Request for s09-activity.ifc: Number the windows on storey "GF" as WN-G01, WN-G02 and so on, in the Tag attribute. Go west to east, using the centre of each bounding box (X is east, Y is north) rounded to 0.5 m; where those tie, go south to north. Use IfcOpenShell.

First a look at what the model holds.

```python
import ifcopenshell
import ifcopenshell.util.element
import ifcopenshell.util.placement

model = ifcopenshell.open("s09-activity.ifc")
print(model.schema)
storey = next(s for s in model.by_type("IfcBuildingStorey") if s.Name == "GF")
windows = [e for e in ifcopenshell.util.element.get_decomposition(storey) if e.is_a("IfcWindow")]
for e in sorted(windows, key=lambda e: e.id()):
    origin = ifcopenshell.util.placement.get_local_placement(e.ObjectPlacement)[:3, 3]
    print(e.id(), e.Tag, e.Name, origin.round(2) + 0.0, sep=" | ")
```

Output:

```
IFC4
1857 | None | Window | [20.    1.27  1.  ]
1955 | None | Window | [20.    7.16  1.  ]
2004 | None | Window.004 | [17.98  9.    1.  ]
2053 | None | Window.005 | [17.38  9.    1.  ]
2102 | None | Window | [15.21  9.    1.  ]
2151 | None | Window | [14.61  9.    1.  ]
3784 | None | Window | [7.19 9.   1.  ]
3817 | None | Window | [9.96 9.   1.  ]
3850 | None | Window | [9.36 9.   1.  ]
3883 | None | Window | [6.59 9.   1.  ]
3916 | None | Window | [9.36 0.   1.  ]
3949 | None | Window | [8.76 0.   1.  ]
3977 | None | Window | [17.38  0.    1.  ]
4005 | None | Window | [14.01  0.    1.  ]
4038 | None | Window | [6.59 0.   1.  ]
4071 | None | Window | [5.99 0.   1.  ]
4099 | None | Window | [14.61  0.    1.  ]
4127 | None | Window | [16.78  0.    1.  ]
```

```python
import ifcopenshell
import ifcopenshell.geom
import ifcopenshell.util.element
import ifcopenshell.util.shape

model = ifcopenshell.open("s09-activity.ifc")
settings = ifcopenshell.geom.settings()
settings.set("use-world-coords", True)


def centre(element):
    shape = ifcopenshell.geom.create_shape(settings, element)
    return ifcopenshell.util.shape.get_bbox_centroid(shape.geometry)


storey = next(s for s in model.by_type("IfcBuildingStorey") if s.Name == "GF")
windows = [e for e in ifcopenshell.util.element.get_decomposition(storey) if e.is_a("IfcWindow")]

# Insertion points can sit at a corner or the storey origin, so sort by the geometry (in metres).
centres = {e: centre(e) for e in windows}
windows.sort(key=lambda e: (round(centres[e][0] / 0.5), centres[e][1]))

for i, e in enumerate(windows, start=1):
    number = f"WN-G{i:02d}"
    e.Tag = number
    print(e.id(), number)

model.write("s09-activity_updated.ifc")
```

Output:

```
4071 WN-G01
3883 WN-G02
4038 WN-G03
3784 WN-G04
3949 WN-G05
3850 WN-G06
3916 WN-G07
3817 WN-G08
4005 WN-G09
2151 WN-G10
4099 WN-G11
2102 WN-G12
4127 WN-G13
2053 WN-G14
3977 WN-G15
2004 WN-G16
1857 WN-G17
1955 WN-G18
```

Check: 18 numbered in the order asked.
